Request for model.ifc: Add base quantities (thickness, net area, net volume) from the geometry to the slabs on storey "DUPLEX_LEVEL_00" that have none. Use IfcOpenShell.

First a look at what the model holds.

```python
import ifcopenshell
import ifcopenshell.util.element
import ifcopenshell.util.unit

model = ifcopenshell.open("model.ifc")
print(model.schema)
for unit_type in ("LENGTHUNIT", "AREAUNIT", "VOLUMEUNIT"):
    print(unit_type, ifcopenshell.util.unit.calculate_unit_scale(model, unit_type))
storey = next(s for s in model.by_type("IfcBuildingStorey") if s.Name == "DUPLEX_LEVEL_00")
slabs = [e for e in ifcopenshell.util.element.get_decomposition(storey) if e.is_a("IfcSlab")]
for e in sorted(slabs, key=lambda e: e.id()):
    print(e.id(), e.is_a(), e.Name, list(ifcopenshell.util.element.get_psets(e, qtos_only=True)), sep=" | ")
```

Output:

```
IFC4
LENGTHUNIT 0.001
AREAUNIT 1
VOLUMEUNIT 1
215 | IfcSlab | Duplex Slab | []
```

```python
import ifcopenshell
import ifcopenshell.api.pset
import ifcopenshell.geom
import ifcopenshell.util.element
import ifcopenshell.util.shape
import ifcopenshell.util.unit

model = ifcopenshell.open("model.ifc")
unit_scale = ifcopenshell.util.unit.calculate_unit_scale(model)
area_scale = ifcopenshell.util.unit.calculate_unit_scale(model, "AREAUNIT")
volume_scale = ifcopenshell.util.unit.calculate_unit_scale(model, "VOLUMEUNIT")
settings = ifcopenshell.geom.settings()

storey = next(s for s in model.by_type("IfcBuildingStorey") if s.Name == "DUPLEX_LEVEL_00")
slabs = [e for e in ifcopenshell.util.element.get_decomposition(storey) if e.is_a("IfcSlab")]

for e in sorted(slabs, key=lambda e: e.id()):
    if ifcopenshell.util.element.get_psets(e, qtos_only=True, should_inherit=False):
        continue
    # Geometry comes back in metres, in the element's own axes.
    shape = ifcopenshell.geom.create_shape(settings, e)
    values = {
        "Width": ifcopenshell.util.shape.get_z(shape.geometry) / unit_scale,
        "NetArea": ifcopenshell.util.shape.get_footprint_area(shape.geometry) / area_scale,
        "NetVolume": ifcopenshell.util.shape.get_volume(shape.geometry) / volume_scale,
    }
    qto = ifcopenshell.api.pset.add_qto(model, product=e, name="Qto_SlabBaseQuantities")
    ifcopenshell.api.pset.edit_qto(model, qto=qto, properties=values)
    print(e.id(), {k: round(v, 3) for k, v in values.items()})

model.write("model_v2.ifc")
```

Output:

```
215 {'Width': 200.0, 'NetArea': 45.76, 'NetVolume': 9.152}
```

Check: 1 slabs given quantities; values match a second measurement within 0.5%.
